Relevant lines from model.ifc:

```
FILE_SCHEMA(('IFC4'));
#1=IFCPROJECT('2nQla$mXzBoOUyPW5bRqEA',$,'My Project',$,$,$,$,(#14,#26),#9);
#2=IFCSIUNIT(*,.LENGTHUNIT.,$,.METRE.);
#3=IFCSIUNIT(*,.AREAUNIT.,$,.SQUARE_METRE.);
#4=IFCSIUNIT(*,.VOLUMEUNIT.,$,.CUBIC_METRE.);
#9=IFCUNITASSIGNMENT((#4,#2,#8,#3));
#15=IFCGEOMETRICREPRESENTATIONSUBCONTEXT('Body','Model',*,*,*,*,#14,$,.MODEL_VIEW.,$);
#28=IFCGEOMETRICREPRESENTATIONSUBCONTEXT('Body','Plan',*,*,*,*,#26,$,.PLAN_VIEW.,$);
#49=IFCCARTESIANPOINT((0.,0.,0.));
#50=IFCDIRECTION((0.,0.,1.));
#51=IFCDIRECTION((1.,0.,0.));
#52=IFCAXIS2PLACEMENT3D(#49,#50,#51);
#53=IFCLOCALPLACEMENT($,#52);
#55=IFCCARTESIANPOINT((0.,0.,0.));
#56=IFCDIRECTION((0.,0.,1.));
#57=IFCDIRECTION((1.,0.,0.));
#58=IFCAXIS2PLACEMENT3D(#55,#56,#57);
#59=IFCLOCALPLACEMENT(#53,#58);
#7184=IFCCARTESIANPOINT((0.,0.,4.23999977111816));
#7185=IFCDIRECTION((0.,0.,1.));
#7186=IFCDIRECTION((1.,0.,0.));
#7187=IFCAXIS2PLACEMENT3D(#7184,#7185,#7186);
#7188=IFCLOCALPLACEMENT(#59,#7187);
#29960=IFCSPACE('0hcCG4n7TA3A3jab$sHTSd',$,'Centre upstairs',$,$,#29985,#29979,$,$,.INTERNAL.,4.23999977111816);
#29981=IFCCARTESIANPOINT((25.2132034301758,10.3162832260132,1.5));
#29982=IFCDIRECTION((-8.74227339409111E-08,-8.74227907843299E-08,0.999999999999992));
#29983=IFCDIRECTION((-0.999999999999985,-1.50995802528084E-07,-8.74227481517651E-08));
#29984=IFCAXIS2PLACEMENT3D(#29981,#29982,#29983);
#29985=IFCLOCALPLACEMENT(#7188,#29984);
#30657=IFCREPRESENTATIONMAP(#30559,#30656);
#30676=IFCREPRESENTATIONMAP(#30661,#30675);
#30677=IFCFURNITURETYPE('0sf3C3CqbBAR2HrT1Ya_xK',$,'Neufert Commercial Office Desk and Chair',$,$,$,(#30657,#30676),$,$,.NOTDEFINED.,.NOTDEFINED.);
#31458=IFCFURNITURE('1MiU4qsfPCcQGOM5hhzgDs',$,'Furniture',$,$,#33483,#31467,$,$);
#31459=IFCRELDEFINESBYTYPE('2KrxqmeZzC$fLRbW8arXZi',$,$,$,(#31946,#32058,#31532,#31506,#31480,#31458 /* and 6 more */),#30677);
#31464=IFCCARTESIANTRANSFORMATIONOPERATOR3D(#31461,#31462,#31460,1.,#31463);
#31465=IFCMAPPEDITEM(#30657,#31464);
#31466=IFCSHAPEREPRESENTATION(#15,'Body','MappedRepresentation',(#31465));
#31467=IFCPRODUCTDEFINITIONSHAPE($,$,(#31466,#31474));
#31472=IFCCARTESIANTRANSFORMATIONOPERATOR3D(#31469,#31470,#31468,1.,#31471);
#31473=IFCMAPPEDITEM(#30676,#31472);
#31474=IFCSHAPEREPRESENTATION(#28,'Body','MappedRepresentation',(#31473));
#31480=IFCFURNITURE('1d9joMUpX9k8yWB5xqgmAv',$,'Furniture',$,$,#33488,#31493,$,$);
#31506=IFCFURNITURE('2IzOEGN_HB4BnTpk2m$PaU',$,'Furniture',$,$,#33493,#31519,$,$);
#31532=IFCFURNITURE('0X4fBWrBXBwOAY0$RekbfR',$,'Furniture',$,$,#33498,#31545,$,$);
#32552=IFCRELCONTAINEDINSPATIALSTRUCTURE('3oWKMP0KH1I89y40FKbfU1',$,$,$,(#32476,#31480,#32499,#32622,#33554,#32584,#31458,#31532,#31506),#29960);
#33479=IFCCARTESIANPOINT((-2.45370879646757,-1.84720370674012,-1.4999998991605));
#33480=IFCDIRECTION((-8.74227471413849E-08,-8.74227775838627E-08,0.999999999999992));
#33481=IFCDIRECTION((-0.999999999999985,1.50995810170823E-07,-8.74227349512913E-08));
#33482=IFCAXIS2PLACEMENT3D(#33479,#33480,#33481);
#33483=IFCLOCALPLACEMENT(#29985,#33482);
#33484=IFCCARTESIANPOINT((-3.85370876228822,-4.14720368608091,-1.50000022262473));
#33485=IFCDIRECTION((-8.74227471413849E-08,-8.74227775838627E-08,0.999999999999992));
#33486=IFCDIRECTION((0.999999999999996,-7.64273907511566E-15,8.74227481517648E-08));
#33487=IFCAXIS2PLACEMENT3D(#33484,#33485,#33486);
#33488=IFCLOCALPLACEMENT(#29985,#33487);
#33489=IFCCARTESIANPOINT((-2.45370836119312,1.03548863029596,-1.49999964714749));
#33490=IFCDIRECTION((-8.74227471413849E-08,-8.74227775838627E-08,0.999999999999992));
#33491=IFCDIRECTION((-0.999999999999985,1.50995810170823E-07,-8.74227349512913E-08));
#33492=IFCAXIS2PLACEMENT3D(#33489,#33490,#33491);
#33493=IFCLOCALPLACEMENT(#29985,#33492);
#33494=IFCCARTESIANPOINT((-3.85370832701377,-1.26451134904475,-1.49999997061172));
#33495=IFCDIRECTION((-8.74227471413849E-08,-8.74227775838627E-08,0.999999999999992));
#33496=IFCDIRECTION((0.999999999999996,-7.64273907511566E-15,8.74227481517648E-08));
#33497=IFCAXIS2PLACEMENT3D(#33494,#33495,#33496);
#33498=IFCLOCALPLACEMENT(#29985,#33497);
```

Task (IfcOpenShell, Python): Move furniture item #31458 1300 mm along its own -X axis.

```python
import ifcopenshell
import ifcopenshell.api.geometry
import ifcopenshell.util.placement

model = ifcopenshell.open("model.ifc")

item = model.by_id(31458)
matrix = ifcopenshell.util.placement.get_local_placement(item.ObjectPlacement)
matrix[:3, 3] -= matrix[:3, 0] * 1.3
ifcopenshell.api.geometry.edit_object_placement(model, product=item, matrix=matrix, is_si=False)

print(ifcopenshell.util.placement.get_local_placement(item.ObjectPlacement).round(3) + 0.0)

model.write("model-out.ifc")
```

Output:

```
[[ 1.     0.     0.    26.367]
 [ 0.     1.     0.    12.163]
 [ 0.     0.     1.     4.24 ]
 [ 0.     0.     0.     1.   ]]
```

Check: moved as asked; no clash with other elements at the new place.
